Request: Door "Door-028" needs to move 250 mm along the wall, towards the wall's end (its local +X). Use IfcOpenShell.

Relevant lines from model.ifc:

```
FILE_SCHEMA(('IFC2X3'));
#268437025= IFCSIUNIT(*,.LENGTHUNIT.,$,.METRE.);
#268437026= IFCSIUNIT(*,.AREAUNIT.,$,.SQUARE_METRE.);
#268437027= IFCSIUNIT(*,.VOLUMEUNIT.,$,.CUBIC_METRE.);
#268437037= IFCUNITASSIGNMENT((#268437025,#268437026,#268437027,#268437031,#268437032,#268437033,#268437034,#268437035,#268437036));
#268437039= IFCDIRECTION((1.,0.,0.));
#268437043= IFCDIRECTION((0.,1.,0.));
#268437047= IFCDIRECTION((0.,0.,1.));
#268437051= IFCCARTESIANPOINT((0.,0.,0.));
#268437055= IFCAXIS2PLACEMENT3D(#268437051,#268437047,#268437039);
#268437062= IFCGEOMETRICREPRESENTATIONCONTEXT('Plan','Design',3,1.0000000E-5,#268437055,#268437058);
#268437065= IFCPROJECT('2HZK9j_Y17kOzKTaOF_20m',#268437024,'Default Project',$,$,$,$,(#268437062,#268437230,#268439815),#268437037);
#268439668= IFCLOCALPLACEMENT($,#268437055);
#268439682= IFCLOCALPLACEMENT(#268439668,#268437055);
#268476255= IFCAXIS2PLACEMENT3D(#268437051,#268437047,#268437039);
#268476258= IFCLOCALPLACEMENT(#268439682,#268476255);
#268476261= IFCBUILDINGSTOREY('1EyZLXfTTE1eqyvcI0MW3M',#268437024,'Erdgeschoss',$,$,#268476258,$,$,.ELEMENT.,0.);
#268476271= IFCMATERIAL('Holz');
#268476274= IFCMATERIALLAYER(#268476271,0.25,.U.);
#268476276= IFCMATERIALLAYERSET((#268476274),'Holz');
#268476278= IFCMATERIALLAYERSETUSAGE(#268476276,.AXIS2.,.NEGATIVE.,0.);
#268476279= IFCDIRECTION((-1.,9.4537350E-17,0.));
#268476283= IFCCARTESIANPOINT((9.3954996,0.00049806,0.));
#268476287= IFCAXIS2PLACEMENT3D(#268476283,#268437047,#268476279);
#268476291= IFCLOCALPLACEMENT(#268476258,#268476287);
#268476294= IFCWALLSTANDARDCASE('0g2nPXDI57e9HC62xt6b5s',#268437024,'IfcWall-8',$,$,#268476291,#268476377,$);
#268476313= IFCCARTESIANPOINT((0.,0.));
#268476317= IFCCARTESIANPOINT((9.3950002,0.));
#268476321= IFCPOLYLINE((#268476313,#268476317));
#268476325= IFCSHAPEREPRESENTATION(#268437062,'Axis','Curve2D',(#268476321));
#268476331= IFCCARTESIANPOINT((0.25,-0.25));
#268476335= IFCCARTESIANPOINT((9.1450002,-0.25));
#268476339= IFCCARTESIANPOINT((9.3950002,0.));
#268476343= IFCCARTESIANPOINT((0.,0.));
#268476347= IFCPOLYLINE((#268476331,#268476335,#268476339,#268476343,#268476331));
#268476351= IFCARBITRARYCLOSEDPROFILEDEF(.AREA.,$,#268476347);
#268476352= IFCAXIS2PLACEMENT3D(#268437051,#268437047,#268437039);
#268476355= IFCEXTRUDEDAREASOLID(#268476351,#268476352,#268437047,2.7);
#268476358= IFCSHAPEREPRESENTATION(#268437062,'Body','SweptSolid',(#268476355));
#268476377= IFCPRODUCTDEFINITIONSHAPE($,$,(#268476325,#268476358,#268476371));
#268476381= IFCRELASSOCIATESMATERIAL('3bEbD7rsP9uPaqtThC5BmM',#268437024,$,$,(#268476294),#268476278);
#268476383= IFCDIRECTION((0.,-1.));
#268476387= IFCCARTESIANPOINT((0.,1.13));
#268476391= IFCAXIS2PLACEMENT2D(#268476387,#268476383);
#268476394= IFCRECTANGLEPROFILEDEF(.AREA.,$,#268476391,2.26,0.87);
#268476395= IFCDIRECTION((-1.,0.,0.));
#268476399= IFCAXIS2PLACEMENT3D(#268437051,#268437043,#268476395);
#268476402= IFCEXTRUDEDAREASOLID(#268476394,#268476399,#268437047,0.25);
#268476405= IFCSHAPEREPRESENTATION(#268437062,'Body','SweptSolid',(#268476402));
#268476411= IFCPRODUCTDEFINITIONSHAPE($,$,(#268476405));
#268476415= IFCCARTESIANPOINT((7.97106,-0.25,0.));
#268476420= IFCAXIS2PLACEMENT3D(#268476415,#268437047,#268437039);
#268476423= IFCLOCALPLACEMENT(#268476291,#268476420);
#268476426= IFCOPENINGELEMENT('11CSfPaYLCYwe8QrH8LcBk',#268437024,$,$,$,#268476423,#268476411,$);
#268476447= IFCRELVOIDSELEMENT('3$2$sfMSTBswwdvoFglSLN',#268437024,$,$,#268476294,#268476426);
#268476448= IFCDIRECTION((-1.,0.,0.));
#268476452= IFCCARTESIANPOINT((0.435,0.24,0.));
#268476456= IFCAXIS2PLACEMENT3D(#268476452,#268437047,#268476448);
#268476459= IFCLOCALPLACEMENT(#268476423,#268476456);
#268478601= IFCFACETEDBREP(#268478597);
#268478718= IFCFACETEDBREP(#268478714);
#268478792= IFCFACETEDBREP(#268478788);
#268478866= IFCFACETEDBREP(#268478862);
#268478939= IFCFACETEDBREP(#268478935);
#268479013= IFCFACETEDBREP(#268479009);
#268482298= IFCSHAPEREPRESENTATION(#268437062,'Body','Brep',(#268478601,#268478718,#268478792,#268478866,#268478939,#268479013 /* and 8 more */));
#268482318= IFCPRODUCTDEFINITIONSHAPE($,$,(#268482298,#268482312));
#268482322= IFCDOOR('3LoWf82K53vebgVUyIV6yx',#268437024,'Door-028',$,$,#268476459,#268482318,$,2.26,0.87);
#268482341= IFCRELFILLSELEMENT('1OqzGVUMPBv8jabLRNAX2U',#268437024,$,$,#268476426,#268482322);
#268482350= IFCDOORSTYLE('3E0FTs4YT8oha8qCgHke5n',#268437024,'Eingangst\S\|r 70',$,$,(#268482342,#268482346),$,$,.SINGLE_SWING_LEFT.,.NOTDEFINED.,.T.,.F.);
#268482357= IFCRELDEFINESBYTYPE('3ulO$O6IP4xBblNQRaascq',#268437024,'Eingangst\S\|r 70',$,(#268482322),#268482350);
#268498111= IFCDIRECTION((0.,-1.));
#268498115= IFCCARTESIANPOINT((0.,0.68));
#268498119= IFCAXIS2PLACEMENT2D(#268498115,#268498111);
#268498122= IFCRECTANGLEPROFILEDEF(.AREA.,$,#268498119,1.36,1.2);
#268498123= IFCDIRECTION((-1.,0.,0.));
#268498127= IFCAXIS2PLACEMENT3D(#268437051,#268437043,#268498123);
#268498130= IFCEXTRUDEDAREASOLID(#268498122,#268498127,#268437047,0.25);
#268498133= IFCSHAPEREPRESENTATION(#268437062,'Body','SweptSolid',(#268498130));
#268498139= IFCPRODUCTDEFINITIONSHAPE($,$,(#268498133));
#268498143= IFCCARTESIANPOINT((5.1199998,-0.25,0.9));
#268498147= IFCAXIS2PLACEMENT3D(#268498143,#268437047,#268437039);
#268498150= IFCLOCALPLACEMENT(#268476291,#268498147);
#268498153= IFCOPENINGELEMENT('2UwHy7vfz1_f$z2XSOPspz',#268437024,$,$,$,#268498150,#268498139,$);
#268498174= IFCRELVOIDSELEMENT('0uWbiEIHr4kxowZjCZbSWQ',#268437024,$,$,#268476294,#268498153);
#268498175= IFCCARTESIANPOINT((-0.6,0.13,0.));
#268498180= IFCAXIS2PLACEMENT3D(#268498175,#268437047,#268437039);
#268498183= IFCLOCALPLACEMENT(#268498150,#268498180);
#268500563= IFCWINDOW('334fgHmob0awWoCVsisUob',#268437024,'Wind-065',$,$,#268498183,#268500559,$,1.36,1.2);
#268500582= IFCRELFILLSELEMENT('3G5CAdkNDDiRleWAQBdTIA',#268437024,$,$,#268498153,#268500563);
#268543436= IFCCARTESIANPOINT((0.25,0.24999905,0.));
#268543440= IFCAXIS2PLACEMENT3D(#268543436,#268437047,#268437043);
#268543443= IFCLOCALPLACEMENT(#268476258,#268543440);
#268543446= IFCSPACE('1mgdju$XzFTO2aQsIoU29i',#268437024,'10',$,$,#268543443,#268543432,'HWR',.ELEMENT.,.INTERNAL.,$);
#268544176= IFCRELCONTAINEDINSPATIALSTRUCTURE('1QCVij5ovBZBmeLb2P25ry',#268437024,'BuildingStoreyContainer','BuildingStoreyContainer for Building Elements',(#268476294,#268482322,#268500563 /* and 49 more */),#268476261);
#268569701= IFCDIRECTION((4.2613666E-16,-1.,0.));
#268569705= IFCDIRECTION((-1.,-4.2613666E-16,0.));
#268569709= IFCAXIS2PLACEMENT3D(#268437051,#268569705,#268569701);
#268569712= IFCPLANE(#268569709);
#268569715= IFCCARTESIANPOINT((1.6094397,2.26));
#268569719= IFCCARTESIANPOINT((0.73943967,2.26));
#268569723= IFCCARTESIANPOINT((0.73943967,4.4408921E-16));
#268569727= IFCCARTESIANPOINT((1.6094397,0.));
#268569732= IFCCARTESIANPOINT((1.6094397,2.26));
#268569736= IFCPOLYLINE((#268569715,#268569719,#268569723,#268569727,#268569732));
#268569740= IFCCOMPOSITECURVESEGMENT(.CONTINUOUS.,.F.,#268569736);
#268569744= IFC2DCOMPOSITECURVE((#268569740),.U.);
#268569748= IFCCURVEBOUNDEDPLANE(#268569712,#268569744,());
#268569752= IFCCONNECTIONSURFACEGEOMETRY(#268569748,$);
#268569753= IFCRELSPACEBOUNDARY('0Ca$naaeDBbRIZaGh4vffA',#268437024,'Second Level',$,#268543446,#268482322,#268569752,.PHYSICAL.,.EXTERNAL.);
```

```python
import numpy as np
import ifcopenshell
import ifcopenshell.api.geometry
import ifcopenshell.util.placement

model = ifcopenshell.open("model.ifc")

door = model.by_guid("3LoWf82K53vebgVUyIV6yx")
opening = door.FillsVoids[0].RelatingOpeningElement
wall = opening.VoidsElements[0].RelatingBuildingElement

wall_matrix = ifcopenshell.util.placement.get_local_placement(wall.ObjectPlacement)
shift = wall_matrix[:3, 0] * 0.25
before = ifcopenshell.util.placement.get_local_placement(door.ObjectPlacement)[:3, 3].copy()

# The door is placed relative to its opening, so it follows when the opening moves.
matrix = ifcopenshell.util.placement.get_local_placement(opening.ObjectPlacement)
matrix[:3, 3] += shift
ifcopenshell.api.geometry.edit_object_placement(
    model, product=opening, matrix=matrix, is_si=False, should_transform_children=True
)

# Space boundary surfaces are stored in each space's coordinates; move them too.
for rel in door.ProvidesBoundaries:
    if not rel.ConnectionGeometry:
        continue
    surface = rel.ConnectionGeometry.SurfaceOnRelatingElement.BasisSurface
    space_matrix = ifcopenshell.util.placement.get_local_placement(rel.RelatingSpace.ObjectPlacement)
    point = np.array(surface.Position.Location.Coordinates) + space_matrix[:3, :3].T @ shift
    surface.Position = model.createIfcAxis2Placement3D(
        model.createIfcCartesianPoint(point.tolist()), surface.Position.Axis, surface.Position.RefDirection
    )

after = ifcopenshell.util.placement.get_local_placement(door.ObjectPlacement)[:3, 3]
print("door moved by", (after - before).round(3) + 0.0)

model.write("model_v2.ifc")
```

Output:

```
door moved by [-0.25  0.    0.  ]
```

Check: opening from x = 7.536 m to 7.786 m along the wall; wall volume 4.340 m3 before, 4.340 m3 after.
